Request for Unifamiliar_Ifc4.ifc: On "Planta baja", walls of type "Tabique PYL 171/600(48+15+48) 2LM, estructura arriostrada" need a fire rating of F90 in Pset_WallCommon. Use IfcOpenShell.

First a look at what the model holds.

```python
import ifcopenshell
import ifcopenshell.util.element

model = ifcopenshell.open("Unifamiliar_Ifc4.ifc")
print(model.schema)
storey = next(s for s in model.by_type("IfcBuildingStorey") if s.Name == "Planta baja")
walls = [e for e in ifcopenshell.util.element.get_decomposition(storey) if e.is_a("IfcWall")]
seen = {}
for e in walls:
    element_type = ifcopenshell.util.element.get_type(e)
    key = (element_type.Name if element_type != e and element_type else None, ifcopenshell.util.element.get_pset(e, "Pset_WallCommon", "FireRating"))
    seen[key] = seen.get(key, 0) + 1
for (name, value), count in sorted(seen.items(), key=str):
    print(count, "x", name, "|", value)
```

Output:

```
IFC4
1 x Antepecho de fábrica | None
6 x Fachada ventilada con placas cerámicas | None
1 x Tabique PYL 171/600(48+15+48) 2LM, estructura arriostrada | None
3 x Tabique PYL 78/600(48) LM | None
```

```python
import ifcopenshell
import ifcopenshell.api.pset
import ifcopenshell.util.element

model = ifcopenshell.open("Unifamiliar_Ifc4.ifc")

storey = next(s for s in model.by_type("IfcBuildingStorey") if s.Name == "Planta baja")
walls = [e for e in ifcopenshell.util.element.get_decomposition(storey) if e.is_a("IfcWall")]

count = 0
for e in walls:
    element_type = ifcopenshell.util.element.get_type(e)
    if element_type in (None, e) or element_type.Name != "Tabique PYL 171/600(48+15+48) 2LM, estructura arriostrada":
        continue
    # add_pset returns the element's existing set when there is one.
    pset = ifcopenshell.api.pset.add_pset(model, product=e, name="Pset_WallCommon")
    ifcopenshell.api.pset.edit_pset(model, pset=pset, properties={"FireRating": "F90"})
    count += 1

print(count, "walls updated")

model.write("Unifamiliar_Ifc4-out.ifc")
```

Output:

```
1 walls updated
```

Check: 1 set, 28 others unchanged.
